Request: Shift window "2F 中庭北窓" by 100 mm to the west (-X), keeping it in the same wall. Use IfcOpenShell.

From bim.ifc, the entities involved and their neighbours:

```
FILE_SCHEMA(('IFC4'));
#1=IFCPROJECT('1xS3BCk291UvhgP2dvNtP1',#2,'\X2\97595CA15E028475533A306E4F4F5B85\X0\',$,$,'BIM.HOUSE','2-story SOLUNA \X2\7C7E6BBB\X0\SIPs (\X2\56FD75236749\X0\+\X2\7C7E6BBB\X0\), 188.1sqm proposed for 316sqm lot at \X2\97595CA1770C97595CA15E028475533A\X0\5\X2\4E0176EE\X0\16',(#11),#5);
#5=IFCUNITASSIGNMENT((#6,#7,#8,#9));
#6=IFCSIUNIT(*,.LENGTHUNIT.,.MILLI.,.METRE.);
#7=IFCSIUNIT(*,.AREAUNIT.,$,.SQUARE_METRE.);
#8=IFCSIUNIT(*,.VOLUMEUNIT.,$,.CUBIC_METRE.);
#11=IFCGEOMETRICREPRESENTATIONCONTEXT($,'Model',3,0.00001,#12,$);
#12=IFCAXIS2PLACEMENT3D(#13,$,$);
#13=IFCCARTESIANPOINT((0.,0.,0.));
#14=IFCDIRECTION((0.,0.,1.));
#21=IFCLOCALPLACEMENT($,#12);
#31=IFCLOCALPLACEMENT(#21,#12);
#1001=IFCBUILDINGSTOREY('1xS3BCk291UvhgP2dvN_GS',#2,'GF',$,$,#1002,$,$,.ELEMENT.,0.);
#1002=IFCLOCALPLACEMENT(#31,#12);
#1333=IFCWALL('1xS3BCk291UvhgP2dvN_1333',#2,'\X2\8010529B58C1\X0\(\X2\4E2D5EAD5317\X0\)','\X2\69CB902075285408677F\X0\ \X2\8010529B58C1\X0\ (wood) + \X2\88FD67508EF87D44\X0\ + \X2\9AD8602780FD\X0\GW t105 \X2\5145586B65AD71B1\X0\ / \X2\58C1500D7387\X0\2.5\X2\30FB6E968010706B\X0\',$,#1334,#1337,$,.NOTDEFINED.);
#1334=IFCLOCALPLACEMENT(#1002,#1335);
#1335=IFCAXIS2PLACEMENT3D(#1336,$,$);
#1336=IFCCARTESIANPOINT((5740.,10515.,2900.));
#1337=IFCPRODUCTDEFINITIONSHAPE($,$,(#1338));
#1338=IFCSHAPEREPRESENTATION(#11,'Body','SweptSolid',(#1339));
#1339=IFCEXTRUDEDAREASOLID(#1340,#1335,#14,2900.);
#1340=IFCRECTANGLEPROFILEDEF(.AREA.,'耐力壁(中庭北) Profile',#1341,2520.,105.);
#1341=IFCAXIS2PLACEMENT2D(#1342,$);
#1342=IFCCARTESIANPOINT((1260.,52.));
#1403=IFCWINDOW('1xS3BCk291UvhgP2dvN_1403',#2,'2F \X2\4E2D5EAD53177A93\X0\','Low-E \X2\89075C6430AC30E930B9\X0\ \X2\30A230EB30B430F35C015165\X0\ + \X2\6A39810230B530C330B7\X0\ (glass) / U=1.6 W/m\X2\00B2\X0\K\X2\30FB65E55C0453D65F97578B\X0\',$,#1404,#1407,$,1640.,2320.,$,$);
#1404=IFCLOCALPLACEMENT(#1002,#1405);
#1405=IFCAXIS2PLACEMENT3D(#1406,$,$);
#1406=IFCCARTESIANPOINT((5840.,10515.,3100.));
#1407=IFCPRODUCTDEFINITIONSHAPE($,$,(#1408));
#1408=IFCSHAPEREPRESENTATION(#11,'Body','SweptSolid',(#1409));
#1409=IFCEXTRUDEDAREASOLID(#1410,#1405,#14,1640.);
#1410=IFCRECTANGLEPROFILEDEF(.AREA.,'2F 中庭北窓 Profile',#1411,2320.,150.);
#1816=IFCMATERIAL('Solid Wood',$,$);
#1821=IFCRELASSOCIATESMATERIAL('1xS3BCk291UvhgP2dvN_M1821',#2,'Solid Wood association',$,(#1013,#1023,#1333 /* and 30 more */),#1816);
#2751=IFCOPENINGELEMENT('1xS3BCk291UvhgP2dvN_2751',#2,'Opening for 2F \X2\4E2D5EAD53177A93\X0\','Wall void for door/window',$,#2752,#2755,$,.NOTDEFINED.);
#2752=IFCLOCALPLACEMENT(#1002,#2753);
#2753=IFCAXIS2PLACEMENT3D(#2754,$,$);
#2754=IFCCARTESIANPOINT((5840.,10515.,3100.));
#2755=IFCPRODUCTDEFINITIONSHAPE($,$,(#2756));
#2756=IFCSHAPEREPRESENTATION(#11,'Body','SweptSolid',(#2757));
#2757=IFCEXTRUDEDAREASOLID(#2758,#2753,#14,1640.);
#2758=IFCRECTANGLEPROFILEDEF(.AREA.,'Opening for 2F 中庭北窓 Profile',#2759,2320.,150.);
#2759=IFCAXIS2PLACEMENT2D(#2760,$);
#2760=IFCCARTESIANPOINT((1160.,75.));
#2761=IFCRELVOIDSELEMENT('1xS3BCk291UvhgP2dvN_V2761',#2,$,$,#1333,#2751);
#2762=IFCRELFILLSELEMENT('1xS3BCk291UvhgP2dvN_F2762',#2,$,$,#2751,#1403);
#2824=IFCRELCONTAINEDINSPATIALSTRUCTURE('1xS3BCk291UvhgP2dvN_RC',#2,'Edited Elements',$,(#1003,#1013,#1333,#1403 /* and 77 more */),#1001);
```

```python
import ifcopenshell
import ifcopenshell.api.geometry
import ifcopenshell.util.placement

model = ifcopenshell.open("bim.ifc")

window = model.by_id(1403)
opening = window.FillsVoids[0].RelatingOpeningElement
wall = opening.VoidsElements[0].RelatingBuildingElement

wall_matrix = ifcopenshell.util.placement.get_local_placement(wall.ObjectPlacement)
shift = wall_matrix[:3, 0] * -100.0
before = ifcopenshell.util.placement.get_local_placement(window.ObjectPlacement)[:3, 3].copy()

# The window is not placed relative to its opening, so move both.
for product in (opening, window):
    matrix = ifcopenshell.util.placement.get_local_placement(product.ObjectPlacement)
    matrix[:3, 3] += shift
    ifcopenshell.api.geometry.edit_object_placement(model, product=product, matrix=matrix, is_si=False)

after = ifcopenshell.util.placement.get_local_placement(window.ObjectPlacement)[:3, 3]
print("window moved by", (after - before).round(3) + 0.0)

model.write("bim-out.ifc")
```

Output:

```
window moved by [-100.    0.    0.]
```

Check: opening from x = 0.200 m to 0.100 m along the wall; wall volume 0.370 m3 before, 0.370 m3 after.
